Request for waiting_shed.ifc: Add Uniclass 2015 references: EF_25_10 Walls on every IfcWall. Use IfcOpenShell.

First a look at what the model holds.

```python
import ifcopenshell

model = ifcopenshell.open("waiting_shed.ifc")
print(model.schema)
print("classifications:", [c.Name for c in model.by_type("IfcClassification")])
for ifc_class in ("IfcDoor", "IfcRoof", "IfcStair", "IfcWall", "IfcWindow"):
    print(ifc_class, len(model.by_type(ifc_class)))
```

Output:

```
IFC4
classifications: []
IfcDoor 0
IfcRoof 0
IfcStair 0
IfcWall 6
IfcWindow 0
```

```python
import ifcopenshell
import ifcopenshell.api.classification

model = ifcopenshell.open("waiting_shed.ifc")

system = ifcopenshell.api.classification.add_classification(model, classification="Uniclass 2015")

codes = {
    "IfcWall": ("EF_25_10", "Walls"),
}
for ifc_class, (code, name) in codes.items():
    products = model.by_type(ifc_class)
    ifcopenshell.api.classification.add_reference(
        model, products=products, classification=system, identification=code, name=name
    )
    print(code, len(products))

model.write("waiting_shed_v2.ifc")
```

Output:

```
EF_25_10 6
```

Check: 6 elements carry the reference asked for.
